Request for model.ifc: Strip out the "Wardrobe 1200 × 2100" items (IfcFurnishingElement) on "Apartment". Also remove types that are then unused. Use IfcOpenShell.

First a look at what the model holds.

```python
import ifcopenshell
import ifcopenshell.util.element

model = ifcopenshell.open("model.ifc")
print(model.schema)
storey = next(s for s in model.by_type("IfcBuildingStorey") if s.Name == "Apartment")
furniture = [e for e in ifcopenshell.util.element.get_decomposition(storey) if e.is_a("IfcFurnishingElement")]
seen = {}
for e in furniture:
    element_type = ifcopenshell.util.element.get_type(e)
    name = element_type.Name if element_type not in (None, e) else None
    seen[name] = seen.get(name, 0) + 1
for name, count in sorted(seen.items(), key=str):
    print(count, "x", name)
```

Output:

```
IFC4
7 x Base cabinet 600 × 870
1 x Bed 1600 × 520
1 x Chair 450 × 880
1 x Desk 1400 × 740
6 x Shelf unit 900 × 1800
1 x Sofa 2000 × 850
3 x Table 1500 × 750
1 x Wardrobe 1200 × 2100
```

```python
import ifcopenshell
import ifcopenshell.api.root
import ifcopenshell.util.element

model = ifcopenshell.open("model.ifc")

storey = next(s for s in model.by_type("IfcBuildingStorey") if s.Name == "Apartment")
furniture = [e for e in ifcopenshell.util.element.get_decomposition(storey) if e.is_a("IfcFurnishingElement")]
targets = [e for e in furniture if (t := ifcopenshell.util.element.get_type(e)) not in (None, e) and t.Name == "Wardrobe 1200 × 2100"]
types = {ifcopenshell.util.element.get_type(e) for e in targets} - {None, *targets}

for e in targets:
    ifcopenshell.api.root.remove_product(model, product=e)
print(len(targets), "removed")

unused = [t for t in types if not ifcopenshell.util.element.get_types(t)]
for t in unused:
    ifcopenshell.api.root.remove_product(model, product=t)
print(len(unused), "unused types removed")

model.write("model_edited.ifc")
```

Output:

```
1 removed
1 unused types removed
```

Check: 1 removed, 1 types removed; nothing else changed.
